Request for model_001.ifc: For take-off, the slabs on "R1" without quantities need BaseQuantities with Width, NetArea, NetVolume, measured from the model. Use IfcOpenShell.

First a look at what the model holds.

```python
import ifcopenshell
import ifcopenshell.util.element
import ifcopenshell.util.unit

model = ifcopenshell.open("model_001.ifc")
print(model.schema)
for unit_type in ("LENGTHUNIT", "AREAUNIT", "VOLUMEUNIT"):
    print(unit_type, ifcopenshell.util.unit.calculate_unit_scale(model, unit_type))
storey = next(s for s in model.by_type("IfcBuildingStorey") if s.Name == "R1")
slabs = [e for e in ifcopenshell.util.element.get_decomposition(storey) if e.is_a("IfcSlab")]
for e in sorted(slabs, key=lambda e: e.id()):
    print(e.id(), e.is_a(), e.Name, list(ifcopenshell.util.element.get_psets(e, qtos_only=True)), sep=" | ")
```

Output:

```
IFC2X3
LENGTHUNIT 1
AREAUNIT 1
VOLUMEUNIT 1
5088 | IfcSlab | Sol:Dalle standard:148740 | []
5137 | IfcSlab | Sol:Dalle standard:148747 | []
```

```python
import ifcopenshell
import ifcopenshell.api.pset
import ifcopenshell.geom
import ifcopenshell.util.element
import ifcopenshell.util.shape
import ifcopenshell.util.unit

model = ifcopenshell.open("model_001.ifc")
unit_scale = ifcopenshell.util.unit.calculate_unit_scale(model)
area_scale = ifcopenshell.util.unit.calculate_unit_scale(model, "AREAUNIT")
volume_scale = ifcopenshell.util.unit.calculate_unit_scale(model, "VOLUMEUNIT")
settings = ifcopenshell.geom.settings()

storey = next(s for s in model.by_type("IfcBuildingStorey") if s.Name == "R1")
slabs = [e for e in ifcopenshell.util.element.get_decomposition(storey) if e.is_a("IfcSlab")]

for e in sorted(slabs, key=lambda e: e.id()):
    if ifcopenshell.util.element.get_psets(e, qtos_only=True, should_inherit=False):
        continue
    # Geometry comes back in metres, in the element's own axes.
    shape = ifcopenshell.geom.create_shape(settings, e)
    values = {
        "Width": ifcopenshell.util.shape.get_z(shape.geometry) / unit_scale,
        "NetArea": ifcopenshell.util.shape.get_footprint_area(shape.geometry) / area_scale,
        "NetVolume": ifcopenshell.util.shape.get_volume(shape.geometry) / volume_scale,
    }
    qto = ifcopenshell.api.pset.add_qto(model, product=e, name="BaseQuantities")
    ifcopenshell.api.pset.edit_qto(model, qto=qto, properties=values)
    print(e.id(), {k: round(v, 3) for k, v in values.items()})

model.write("model_001_v2.ifc")
```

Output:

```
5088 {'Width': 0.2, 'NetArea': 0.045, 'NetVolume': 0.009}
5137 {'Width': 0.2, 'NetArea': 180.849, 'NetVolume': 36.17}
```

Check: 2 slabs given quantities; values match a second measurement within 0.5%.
